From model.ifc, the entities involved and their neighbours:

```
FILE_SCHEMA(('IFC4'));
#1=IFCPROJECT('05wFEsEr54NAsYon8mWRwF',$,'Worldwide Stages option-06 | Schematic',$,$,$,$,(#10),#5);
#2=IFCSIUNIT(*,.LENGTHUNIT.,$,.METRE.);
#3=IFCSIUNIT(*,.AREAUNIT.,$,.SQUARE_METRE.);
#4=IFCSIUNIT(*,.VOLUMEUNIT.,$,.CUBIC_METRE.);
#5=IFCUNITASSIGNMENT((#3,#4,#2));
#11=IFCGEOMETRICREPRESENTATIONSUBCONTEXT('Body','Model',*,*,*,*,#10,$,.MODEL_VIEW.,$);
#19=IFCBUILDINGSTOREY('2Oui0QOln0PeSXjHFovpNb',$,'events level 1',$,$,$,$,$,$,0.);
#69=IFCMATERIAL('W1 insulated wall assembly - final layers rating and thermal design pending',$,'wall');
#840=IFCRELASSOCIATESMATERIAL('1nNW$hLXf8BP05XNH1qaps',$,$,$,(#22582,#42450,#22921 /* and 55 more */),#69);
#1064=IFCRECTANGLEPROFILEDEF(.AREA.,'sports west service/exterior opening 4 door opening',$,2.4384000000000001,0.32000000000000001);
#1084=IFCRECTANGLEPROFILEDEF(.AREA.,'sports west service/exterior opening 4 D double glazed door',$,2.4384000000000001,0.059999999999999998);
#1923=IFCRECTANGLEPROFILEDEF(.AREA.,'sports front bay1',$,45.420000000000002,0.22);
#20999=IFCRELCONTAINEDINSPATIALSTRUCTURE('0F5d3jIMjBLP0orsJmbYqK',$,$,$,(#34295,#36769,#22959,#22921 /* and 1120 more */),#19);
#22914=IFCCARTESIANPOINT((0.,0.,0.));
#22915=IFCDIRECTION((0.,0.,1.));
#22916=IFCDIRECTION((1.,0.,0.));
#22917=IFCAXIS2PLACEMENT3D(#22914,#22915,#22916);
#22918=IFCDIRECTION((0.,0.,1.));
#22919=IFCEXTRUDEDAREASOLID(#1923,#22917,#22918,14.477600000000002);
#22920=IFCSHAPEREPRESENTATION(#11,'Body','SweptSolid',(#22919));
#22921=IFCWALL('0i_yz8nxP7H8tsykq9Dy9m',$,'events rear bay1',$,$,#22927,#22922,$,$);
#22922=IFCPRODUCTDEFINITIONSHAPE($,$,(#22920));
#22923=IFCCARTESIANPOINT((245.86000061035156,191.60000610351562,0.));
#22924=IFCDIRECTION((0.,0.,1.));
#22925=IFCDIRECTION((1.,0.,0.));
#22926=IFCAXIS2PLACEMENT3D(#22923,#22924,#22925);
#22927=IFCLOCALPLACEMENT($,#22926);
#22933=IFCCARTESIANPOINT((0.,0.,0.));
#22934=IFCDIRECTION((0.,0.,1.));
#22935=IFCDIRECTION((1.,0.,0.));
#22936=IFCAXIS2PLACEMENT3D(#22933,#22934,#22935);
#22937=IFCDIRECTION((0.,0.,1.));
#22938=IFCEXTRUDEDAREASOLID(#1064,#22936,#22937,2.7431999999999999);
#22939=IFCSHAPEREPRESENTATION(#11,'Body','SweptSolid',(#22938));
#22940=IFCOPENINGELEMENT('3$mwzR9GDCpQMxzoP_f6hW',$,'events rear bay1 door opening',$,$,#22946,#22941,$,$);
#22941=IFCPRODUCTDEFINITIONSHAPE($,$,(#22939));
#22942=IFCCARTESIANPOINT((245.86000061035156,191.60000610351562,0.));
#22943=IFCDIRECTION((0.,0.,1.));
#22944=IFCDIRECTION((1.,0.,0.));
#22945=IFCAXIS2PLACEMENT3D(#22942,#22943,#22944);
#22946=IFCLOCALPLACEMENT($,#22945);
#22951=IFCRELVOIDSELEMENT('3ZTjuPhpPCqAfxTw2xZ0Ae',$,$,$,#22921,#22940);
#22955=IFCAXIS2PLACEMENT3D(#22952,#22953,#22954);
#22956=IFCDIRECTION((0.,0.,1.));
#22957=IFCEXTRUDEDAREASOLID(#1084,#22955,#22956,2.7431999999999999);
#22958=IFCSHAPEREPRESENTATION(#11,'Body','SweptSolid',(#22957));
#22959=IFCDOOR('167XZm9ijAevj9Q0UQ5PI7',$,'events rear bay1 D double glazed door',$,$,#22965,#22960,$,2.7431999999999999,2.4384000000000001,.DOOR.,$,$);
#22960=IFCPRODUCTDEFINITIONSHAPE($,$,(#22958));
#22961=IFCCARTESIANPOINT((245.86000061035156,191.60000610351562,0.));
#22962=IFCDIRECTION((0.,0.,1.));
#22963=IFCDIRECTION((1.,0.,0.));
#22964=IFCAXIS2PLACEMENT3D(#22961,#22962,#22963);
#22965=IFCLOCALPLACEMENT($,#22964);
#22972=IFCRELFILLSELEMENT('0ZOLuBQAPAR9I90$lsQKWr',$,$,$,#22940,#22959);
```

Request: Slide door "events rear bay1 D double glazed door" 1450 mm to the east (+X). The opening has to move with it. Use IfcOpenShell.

```python
import ifcopenshell
import ifcopenshell.api.geometry
import ifcopenshell.util.placement
import ifcopenshell.util.unit

model = ifcopenshell.open("model.ifc")
unit_scale = ifcopenshell.util.unit.calculate_unit_scale(model)

door = model.by_guid("167XZm9ijAevj9Q0UQ5PI7")
opening = door.FillsVoids[0].RelatingOpeningElement
wall = opening.VoidsElements[0].RelatingBuildingElement

wall_matrix = ifcopenshell.util.placement.get_local_placement(wall.ObjectPlacement)
shift = wall_matrix[:3, 0] * 1.45 / unit_scale
before = ifcopenshell.util.placement.get_local_placement(door.ObjectPlacement)[:3, 3].copy()

# The door is not placed relative to its opening, so move both.
for product in (opening, door):
    matrix = ifcopenshell.util.placement.get_local_placement(product.ObjectPlacement)
    matrix[:3, 3] += shift
    ifcopenshell.api.geometry.edit_object_placement(model, product=product, matrix=matrix, is_si=False)

after = ifcopenshell.util.placement.get_local_placement(door.ObjectPlacement)[:3, 3]
print("door moved by", (after - before).round(3) + 0.0)

model.write("model_edited.ifc")
```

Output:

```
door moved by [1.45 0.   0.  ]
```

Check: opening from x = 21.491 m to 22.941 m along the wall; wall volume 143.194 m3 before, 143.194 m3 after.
